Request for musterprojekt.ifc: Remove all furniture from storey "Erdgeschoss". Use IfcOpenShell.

First a look at what the model holds.

```python
import ifcopenshell
import ifcopenshell.util.element

model = ifcopenshell.open("musterprojekt.ifc")
print(model.schema)
storey = next(s for s in model.by_type("IfcBuildingStorey") if s.Name == "Erdgeschoss")
furniture = [e for e in ifcopenshell.util.element.get_decomposition(storey) if e.is_a("IfcFurnishingElement")]
seen = {}
for e in furniture:
    element_type = ifcopenshell.util.element.get_type(e)
    name = element_type.Name if element_type not in (None, e) else None
    seen[name] = seen.get(name, 0) + 1
for name, count in sorted(seen.items(), key=str):
    print(count, "x", name)
```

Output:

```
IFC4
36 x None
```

```python
import ifcopenshell
import ifcopenshell.api.root
import ifcopenshell.util.element

model = ifcopenshell.open("musterprojekt.ifc")

storey = next(s for s in model.by_type("IfcBuildingStorey") if s.Name == "Erdgeschoss")
furniture = [e for e in ifcopenshell.util.element.get_decomposition(storey) if e.is_a("IfcFurnishingElement")]

for e in furniture:
    ifcopenshell.api.root.remove_product(model, product=e)
print(len(furniture), "removed")

model.write("musterprojekt_v2.ifc")
```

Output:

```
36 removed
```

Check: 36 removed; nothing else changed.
